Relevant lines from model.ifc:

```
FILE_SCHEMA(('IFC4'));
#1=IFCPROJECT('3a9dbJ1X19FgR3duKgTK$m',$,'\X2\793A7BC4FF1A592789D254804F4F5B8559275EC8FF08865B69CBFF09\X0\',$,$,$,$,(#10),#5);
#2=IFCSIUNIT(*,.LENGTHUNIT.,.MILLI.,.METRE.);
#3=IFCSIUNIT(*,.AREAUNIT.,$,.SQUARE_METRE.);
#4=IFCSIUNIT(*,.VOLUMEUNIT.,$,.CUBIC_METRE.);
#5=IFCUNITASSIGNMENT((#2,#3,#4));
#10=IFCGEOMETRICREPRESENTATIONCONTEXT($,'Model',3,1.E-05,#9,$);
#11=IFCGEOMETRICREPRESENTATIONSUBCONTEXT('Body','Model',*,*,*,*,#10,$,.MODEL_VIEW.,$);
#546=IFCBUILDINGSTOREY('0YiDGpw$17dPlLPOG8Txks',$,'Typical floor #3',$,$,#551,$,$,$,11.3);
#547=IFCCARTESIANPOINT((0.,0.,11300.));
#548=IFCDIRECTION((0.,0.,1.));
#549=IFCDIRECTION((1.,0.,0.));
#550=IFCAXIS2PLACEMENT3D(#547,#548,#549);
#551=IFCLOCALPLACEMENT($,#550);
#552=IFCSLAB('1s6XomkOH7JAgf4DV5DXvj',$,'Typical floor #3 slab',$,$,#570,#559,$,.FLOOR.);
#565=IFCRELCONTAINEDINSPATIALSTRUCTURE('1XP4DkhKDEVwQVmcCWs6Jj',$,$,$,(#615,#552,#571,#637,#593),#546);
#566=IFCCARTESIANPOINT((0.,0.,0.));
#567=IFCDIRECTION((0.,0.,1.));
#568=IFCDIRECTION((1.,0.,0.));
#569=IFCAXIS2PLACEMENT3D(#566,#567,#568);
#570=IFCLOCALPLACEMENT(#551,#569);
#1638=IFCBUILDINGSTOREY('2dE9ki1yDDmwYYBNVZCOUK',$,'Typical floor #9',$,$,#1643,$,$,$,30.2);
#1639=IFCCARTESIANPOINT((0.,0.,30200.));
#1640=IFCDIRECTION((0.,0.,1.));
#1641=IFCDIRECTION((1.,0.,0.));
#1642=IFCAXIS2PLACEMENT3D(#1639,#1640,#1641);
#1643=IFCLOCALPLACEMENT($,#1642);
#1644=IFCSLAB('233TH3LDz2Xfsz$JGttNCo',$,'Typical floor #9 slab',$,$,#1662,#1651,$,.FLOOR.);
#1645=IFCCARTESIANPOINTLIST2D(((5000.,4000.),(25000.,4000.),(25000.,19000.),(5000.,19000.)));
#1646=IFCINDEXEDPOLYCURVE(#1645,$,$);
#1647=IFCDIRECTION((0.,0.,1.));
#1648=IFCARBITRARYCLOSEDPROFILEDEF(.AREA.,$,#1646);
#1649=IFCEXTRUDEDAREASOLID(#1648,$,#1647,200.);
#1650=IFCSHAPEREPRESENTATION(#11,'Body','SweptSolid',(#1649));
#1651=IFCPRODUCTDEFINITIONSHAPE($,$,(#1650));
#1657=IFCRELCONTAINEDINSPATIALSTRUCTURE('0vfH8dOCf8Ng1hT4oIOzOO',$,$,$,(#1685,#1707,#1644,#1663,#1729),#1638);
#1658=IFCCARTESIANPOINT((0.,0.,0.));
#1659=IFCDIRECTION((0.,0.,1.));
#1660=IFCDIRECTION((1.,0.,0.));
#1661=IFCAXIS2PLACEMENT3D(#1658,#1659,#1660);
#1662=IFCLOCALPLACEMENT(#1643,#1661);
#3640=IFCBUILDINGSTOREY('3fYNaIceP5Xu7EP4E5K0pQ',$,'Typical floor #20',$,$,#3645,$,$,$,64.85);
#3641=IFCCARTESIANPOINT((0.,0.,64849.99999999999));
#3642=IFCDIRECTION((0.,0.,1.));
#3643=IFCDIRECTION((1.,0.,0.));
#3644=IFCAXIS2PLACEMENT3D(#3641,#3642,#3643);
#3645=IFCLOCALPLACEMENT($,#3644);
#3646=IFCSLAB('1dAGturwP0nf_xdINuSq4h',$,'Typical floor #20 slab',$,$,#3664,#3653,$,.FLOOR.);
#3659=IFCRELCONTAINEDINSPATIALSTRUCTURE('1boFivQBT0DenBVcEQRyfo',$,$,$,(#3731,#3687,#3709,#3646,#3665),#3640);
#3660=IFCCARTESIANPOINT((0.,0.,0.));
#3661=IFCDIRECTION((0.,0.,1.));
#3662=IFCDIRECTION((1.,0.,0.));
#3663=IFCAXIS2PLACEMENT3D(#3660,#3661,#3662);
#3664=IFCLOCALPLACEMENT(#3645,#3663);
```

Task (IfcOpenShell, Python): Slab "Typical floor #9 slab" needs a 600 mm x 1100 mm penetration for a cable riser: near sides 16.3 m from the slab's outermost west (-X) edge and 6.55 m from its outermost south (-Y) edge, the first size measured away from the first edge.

```python
import numpy as np
import ifcopenshell
import ifcopenshell.api.feature
import ifcopenshell.api.geometry
import ifcopenshell.api.root
import ifcopenshell.geom
import ifcopenshell.util.placement
import ifcopenshell.util.representation
import ifcopenshell.util.shape
import ifcopenshell.util.unit

model = ifcopenshell.open("model.ifc")
unit_scale = ifcopenshell.util.unit.calculate_unit_scale(model)
settings = ifcopenshell.geom.settings()


def volume(element):
    """Net volume in cubic metres, openings subtracted."""
    shape = ifcopenshell.geom.create_shape(settings, element)
    return ifcopenshell.util.shape.get_volume(shape.geometry)


slab = model.by_id(1644)
before = volume(slab)

# Extent in the slab's own axes, in metres. The edges named are its -X and -Y sides.
slab_shape = ifcopenshell.geom.create_shape(settings, slab)
vertices = ifcopenshell.util.shape.get_vertices(slab_shape.geometry)
x_min, y_min, bottom = vertices.min(axis=0)
top = vertices[:, 2].max()

opening = ifcopenshell.api.root.create_entity(model, ifc_class="IfcOpeningElement", name="Cable riser opening", predefined_type="OPENING")
context = ifcopenshell.util.representation.get_context(model, "Model", "Body", "MODEL_VIEW")
width, depth = 0.6, 1.1
outline = [(0.0, 0.0), (width, 0.0), (width, depth), (0.0, depth), (0.0, 0.0)]
# Overshoot both faces by 50 mm so the cut is clean.
shape = ifcopenshell.api.geometry.add_slab_representation(
    model, context=context, depth=top - bottom + 0.1, polyline=outline
)
ifcopenshell.api.geometry.assign_representation(model, product=opening, representation=shape)

matrix = ifcopenshell.util.placement.get_local_placement(slab.ObjectPlacement)
matrix[:, 3] = matrix @ np.append(np.array([x_min + 16.3, y_min + 6.55, bottom - 0.05]) / unit_scale, 1.0)
ifcopenshell.api.geometry.edit_object_placement(model, product=opening, matrix=matrix, is_si=False)
ifcopenshell.api.feature.add_feature(model, feature=opening, element=slab)

after = volume(slab)

print(f"slab volume {before:.3f} -> {after:.3f} m3")

model.write("model_updated.ifc")
```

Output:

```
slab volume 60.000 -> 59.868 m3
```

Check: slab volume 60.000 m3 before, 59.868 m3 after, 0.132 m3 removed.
